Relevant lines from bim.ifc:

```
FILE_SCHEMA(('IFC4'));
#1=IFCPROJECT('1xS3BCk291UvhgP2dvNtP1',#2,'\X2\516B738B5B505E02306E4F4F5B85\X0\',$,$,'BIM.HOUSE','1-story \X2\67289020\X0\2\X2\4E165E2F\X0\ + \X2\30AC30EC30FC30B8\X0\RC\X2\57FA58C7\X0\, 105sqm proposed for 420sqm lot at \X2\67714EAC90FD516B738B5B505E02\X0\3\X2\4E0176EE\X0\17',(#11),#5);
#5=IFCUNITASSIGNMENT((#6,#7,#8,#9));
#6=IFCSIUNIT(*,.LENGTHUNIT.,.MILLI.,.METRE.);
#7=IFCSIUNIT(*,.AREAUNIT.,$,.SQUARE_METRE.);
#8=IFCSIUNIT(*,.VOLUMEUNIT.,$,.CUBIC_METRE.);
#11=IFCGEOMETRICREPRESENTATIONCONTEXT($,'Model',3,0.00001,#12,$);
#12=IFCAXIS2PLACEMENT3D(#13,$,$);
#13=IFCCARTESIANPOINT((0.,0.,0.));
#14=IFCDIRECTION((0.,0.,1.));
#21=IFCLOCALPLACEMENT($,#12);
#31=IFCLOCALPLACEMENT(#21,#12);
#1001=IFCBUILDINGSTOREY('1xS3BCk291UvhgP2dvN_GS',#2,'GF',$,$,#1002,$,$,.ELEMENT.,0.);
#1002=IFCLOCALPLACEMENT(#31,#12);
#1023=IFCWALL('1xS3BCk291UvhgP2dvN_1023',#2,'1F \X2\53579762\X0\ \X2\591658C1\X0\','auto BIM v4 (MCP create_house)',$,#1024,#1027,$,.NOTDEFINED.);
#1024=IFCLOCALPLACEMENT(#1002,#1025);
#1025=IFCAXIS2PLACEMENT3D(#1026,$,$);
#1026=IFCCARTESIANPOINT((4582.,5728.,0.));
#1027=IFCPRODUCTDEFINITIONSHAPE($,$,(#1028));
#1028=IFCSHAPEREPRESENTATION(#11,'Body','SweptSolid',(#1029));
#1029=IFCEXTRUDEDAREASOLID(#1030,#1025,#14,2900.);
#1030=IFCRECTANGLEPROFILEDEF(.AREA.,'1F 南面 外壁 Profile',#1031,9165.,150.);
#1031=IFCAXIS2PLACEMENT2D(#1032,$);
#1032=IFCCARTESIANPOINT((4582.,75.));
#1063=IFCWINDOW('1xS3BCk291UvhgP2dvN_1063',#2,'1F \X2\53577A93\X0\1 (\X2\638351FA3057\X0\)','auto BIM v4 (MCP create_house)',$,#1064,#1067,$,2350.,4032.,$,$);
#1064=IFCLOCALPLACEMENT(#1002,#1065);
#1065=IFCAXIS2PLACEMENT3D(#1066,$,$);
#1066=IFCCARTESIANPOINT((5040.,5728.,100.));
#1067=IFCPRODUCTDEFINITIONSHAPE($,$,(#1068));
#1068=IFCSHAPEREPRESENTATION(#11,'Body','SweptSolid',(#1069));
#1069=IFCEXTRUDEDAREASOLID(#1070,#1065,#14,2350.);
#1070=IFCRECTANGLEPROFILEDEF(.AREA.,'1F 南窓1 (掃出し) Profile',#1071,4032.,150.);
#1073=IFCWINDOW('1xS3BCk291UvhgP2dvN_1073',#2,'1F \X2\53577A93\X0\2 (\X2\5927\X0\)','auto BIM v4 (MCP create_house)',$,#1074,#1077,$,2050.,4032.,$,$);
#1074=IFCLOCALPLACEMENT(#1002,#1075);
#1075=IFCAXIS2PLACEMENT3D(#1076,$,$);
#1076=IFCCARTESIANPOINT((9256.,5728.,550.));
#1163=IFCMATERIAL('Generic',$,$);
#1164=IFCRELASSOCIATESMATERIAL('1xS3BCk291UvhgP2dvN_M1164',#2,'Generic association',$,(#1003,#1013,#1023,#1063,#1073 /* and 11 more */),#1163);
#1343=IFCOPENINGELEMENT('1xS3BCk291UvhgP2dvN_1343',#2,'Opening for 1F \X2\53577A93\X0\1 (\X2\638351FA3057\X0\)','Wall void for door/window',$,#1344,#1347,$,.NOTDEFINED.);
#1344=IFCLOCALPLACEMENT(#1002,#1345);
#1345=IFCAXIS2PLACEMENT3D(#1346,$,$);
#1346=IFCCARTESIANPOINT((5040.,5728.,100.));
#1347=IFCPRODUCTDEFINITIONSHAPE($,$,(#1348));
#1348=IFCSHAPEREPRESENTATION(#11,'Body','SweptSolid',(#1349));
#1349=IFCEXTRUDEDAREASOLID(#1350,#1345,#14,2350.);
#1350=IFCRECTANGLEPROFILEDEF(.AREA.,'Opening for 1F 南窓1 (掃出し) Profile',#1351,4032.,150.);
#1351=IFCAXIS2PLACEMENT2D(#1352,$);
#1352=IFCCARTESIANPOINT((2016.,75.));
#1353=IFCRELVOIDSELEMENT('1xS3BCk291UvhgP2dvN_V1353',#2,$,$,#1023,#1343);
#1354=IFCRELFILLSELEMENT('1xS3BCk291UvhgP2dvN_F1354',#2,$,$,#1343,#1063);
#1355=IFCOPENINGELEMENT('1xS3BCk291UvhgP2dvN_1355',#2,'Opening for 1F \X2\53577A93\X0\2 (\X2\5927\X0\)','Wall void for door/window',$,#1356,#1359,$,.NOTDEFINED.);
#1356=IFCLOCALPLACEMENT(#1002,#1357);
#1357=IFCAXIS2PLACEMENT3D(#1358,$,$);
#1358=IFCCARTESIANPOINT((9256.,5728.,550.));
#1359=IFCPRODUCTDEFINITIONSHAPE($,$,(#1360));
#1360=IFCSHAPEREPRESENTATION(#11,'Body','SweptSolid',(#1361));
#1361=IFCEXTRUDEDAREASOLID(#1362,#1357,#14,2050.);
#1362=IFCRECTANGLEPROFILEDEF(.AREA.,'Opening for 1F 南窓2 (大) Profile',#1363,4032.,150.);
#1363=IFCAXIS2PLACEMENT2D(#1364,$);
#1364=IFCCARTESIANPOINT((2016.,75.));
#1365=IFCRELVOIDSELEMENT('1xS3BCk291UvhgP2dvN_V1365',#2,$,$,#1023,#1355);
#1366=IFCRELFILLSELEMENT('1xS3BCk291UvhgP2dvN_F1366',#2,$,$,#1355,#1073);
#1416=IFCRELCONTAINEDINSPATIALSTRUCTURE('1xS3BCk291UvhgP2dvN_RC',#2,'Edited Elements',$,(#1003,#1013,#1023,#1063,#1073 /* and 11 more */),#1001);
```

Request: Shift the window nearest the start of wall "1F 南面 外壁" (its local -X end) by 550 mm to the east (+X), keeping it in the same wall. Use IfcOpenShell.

```python
import ifcopenshell
import ifcopenshell.api.geometry
import ifcopenshell.util.placement
import ifcopenshell.util.unit

model = ifcopenshell.open("bim.ifc")
unit_scale = ifcopenshell.util.unit.calculate_unit_scale(model)

window = model.by_guid("1xS3BCk291UvhgP2dvN_1063")
opening = window.FillsVoids[0].RelatingOpeningElement
wall = opening.VoidsElements[0].RelatingBuildingElement

wall_matrix = ifcopenshell.util.placement.get_local_placement(wall.ObjectPlacement)
shift = wall_matrix[:3, 0] * 0.55 / unit_scale
before = ifcopenshell.util.placement.get_local_placement(window.ObjectPlacement)[:3, 3].copy()

# The window is not placed relative to its opening, so move both.
for product in (opening, window):
    matrix = ifcopenshell.util.placement.get_local_placement(product.ObjectPlacement)
    matrix[:3, 3] += shift
    ifcopenshell.api.geometry.edit_object_placement(model, product=product, matrix=matrix, is_si=False)

after = ifcopenshell.util.placement.get_local_placement(window.ObjectPlacement)[:3, 3]
print("window moved by", (after - before).round(3) + 0.0)

model.write("bim_v2.ifc")
```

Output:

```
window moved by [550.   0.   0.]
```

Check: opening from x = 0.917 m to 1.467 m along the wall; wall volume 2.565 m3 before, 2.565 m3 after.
